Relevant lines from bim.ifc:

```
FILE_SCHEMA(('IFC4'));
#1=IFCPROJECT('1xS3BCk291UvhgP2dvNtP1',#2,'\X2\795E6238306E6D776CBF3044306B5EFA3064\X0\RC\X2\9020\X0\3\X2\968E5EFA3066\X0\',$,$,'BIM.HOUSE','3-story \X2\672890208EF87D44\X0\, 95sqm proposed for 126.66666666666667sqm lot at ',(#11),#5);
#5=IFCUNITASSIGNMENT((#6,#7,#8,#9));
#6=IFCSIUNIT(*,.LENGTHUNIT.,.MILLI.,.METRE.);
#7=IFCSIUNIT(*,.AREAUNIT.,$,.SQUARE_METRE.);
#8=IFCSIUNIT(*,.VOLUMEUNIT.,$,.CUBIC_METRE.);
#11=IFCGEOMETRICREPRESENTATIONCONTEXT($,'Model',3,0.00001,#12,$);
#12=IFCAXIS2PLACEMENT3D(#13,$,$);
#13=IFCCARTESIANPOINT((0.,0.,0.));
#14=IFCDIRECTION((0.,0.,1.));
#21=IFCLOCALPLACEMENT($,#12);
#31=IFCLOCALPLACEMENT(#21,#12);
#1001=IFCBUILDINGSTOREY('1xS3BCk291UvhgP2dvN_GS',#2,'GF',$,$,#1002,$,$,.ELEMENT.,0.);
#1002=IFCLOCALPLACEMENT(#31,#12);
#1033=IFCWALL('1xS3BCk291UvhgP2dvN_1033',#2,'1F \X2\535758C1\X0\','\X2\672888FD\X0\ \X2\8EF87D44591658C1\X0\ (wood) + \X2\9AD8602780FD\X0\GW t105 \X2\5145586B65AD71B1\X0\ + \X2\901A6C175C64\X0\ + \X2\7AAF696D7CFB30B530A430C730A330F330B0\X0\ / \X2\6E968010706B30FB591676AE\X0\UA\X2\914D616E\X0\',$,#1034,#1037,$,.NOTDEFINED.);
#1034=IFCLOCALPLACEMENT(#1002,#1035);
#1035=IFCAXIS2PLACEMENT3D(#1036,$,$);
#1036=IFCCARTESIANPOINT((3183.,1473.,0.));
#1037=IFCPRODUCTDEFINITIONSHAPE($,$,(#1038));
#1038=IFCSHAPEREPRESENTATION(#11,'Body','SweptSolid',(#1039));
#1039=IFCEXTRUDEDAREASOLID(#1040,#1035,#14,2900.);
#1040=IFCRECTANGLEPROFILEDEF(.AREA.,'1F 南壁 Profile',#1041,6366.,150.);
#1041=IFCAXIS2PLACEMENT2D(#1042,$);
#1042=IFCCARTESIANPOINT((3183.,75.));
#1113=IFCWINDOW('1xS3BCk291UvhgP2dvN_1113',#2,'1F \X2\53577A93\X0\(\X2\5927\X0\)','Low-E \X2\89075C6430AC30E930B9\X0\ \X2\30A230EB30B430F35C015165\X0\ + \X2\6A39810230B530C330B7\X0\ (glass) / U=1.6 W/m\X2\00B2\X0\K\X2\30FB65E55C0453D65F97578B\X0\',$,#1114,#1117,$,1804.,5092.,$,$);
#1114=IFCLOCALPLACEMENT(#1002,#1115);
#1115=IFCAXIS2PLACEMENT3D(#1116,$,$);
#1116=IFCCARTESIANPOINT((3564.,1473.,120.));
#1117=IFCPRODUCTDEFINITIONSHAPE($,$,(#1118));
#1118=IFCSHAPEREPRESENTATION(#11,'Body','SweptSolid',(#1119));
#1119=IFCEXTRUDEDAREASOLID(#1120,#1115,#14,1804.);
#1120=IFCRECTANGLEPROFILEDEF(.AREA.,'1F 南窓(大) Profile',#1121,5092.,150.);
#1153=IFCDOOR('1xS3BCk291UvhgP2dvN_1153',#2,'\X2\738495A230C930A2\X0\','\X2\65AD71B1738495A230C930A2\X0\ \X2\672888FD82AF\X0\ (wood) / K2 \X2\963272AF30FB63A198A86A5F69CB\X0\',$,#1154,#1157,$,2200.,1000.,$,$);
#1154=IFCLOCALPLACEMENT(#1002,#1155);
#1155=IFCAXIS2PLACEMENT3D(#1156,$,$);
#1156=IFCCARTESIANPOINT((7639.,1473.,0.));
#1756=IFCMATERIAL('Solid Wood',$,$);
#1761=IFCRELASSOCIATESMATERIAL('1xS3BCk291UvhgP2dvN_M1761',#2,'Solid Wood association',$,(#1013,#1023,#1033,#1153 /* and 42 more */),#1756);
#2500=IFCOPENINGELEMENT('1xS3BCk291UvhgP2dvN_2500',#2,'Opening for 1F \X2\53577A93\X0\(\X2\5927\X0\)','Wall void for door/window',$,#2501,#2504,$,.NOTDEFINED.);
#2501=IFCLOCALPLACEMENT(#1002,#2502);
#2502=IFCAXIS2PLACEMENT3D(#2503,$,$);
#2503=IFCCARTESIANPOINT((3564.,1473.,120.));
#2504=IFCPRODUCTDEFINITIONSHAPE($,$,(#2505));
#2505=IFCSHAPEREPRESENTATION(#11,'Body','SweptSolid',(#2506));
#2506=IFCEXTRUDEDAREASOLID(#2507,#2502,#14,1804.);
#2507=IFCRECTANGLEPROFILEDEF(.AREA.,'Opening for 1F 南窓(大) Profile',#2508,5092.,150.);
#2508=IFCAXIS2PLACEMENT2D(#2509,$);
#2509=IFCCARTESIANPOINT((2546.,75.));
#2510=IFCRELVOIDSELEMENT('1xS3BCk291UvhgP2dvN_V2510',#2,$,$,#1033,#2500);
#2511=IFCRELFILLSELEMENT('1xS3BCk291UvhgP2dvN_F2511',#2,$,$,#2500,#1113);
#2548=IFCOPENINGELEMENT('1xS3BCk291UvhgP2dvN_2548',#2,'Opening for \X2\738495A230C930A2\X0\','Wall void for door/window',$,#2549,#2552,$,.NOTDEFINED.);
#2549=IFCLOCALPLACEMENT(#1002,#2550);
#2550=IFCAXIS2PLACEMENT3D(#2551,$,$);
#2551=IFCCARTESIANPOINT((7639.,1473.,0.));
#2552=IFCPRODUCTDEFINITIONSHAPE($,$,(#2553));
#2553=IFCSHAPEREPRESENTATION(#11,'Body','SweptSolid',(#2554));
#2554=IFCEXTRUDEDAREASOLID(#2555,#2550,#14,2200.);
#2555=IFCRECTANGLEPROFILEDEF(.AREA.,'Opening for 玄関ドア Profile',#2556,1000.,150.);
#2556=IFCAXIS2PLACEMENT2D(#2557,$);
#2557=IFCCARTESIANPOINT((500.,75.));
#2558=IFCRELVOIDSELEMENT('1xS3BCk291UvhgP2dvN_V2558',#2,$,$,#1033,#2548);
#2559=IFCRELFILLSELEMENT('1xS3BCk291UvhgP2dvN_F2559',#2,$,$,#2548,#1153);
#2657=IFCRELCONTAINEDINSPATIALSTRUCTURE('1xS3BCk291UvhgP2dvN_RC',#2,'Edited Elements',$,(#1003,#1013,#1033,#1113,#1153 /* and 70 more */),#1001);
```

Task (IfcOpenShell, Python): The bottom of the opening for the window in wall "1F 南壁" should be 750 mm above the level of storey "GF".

```python
import numpy as np
import ifcopenshell
import ifcopenshell.api.geometry
import ifcopenshell.geom
import ifcopenshell.util.element
import ifcopenshell.util.placement
import ifcopenshell.util.shape
import ifcopenshell.util.unit

model = ifcopenshell.open("bim.ifc")
unit_scale = ifcopenshell.util.unit.calculate_unit_scale(model)

window = model.by_guid("1xS3BCk291UvhgP2dvN_1113")
opening = window.FillsVoids[0].RelatingOpeningElement
storey = ifcopenshell.util.element.get_container(window, ifc_class="IfcBuildingStorey")
level = ifcopenshell.util.placement.get_local_placement(storey.ObjectPlacement)[2, 3]

# The opening's origin need not be at the sill, so measure its lowest point.
shape = ifcopenshell.geom.create_shape(ifcopenshell.geom.settings(), opening)
bottom = ifcopenshell.util.shape.get_shape_bottom_elevation(shape, shape.geometry) / unit_scale
dz = level + 0.75 / unit_scale - bottom

shift = np.array([0.0, 0.0, dz])
# The window is not placed relative to its opening, so move both.
for product in (opening, window):
    matrix = ifcopenshell.util.placement.get_local_placement(product.ObjectPlacement)
    matrix[:3, 3] += shift
    ifcopenshell.api.geometry.edit_object_placement(model, product=product, matrix=matrix, is_si=False)

print(f"moved by {dz * unit_scale:+.3f} m")

model.write("bim-out.ifc")
```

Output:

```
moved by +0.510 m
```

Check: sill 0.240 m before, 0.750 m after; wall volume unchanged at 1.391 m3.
